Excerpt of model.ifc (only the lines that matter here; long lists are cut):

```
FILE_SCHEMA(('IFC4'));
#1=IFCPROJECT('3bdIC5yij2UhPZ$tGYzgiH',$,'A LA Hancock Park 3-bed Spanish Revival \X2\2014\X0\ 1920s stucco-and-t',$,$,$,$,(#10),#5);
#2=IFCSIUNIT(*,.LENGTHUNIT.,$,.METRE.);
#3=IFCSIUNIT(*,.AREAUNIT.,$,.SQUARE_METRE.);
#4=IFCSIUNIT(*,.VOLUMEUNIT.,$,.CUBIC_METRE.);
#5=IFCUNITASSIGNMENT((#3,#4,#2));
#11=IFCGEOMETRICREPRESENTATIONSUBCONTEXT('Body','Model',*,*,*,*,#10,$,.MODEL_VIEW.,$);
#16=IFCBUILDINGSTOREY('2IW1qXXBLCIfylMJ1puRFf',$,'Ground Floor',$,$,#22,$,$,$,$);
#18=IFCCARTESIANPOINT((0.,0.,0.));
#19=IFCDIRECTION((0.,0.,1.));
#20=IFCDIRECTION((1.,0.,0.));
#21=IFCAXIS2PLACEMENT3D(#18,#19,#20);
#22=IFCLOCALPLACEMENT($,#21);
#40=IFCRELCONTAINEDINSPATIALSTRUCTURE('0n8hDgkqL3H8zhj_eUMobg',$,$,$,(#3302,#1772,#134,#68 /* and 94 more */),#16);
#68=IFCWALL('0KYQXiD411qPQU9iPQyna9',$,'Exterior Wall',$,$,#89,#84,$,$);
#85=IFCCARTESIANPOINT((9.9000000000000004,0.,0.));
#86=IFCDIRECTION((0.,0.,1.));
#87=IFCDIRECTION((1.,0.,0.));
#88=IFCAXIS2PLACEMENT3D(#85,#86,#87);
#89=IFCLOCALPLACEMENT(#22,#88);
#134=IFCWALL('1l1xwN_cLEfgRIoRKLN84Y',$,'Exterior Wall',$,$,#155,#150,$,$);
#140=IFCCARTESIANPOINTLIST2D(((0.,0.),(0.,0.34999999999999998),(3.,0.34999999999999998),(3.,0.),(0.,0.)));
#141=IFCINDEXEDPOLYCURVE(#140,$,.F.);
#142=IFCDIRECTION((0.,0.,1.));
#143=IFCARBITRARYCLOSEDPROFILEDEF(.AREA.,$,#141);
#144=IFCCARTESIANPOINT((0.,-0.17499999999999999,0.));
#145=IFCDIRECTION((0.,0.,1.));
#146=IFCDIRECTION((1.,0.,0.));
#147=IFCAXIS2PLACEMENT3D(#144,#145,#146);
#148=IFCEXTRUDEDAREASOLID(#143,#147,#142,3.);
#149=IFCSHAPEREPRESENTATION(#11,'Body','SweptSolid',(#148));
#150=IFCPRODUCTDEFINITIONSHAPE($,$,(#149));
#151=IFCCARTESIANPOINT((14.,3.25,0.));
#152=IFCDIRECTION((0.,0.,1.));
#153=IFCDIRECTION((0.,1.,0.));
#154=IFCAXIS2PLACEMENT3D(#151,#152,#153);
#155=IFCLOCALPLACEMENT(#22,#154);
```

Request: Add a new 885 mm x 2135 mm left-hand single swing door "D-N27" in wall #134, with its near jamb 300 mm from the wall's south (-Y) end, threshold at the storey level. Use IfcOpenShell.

```python
import numpy as np
import ifcopenshell
import ifcopenshell.api.feature
import ifcopenshell.api.geometry
import ifcopenshell.api.root
import ifcopenshell.api.spatial
import ifcopenshell.geom
import ifcopenshell.util.element
import ifcopenshell.util.placement
import ifcopenshell.util.representation
import ifcopenshell.util.shape
import ifcopenshell.util.unit

model = ifcopenshell.open("model.ifc")
unit_scale = ifcopenshell.util.unit.calculate_unit_scale(model)
settings = ifcopenshell.geom.settings()


def volume(element):
    """Net volume in cubic metres, openings subtracted."""
    shape = ifcopenshell.geom.create_shape(settings, element)
    return ifcopenshell.util.shape.get_volume(shape.geometry)


wall = model.by_guid("1l1xwN_cLEfgRIoRKLN84Y")
storey = ifcopenshell.util.element.get_container(wall, ifc_class="IfcBuildingStorey")
context = ifcopenshell.util.representation.get_context(model, "Model", "Body", "MODEL_VIEW")
before = volume(wall)

width, height, from_end, sill = 0.885, 2.135, 0.3, 0.0  # metres

# The wall runs along its own X axis, and the end named is its -X end.
wall_shape = ifcopenshell.geom.create_shape(settings, wall)
x, y, z = ifcopenshell.util.shape.get_vertices(wall_shape.geometry).T
start = x.min() + from_end
face, thickness = float(y.min()), float(y.max() - y.min())
wall_matrix = ifcopenshell.util.placement.get_local_placement(wall.ObjectPlacement)
level = ifcopenshell.util.placement.get_local_placement(storey.ObjectPlacement)[2, 3]


def in_wall(x, y):
    """Placement at x, y metres in the wall's axes, at sill height."""
    matrix = wall_matrix.copy()
    matrix[:, 3] = wall_matrix @ np.array([x / unit_scale, y / unit_scale, 0.0, 1.0])
    matrix[2, 3] = level + sill / unit_scale
    return matrix


# Opening: a box that overshoots both wall faces by 50 mm.
opening = ifcopenshell.api.root.create_entity(model, ifc_class="IfcOpeningElement", predefined_type="OPENING")
box = ifcopenshell.api.geometry.add_wall_representation(
    model, context=context, length=width, height=height, thickness=thickness + 0.1
)
ifcopenshell.api.geometry.assign_representation(model, product=opening, representation=box)
ifcopenshell.api.geometry.edit_object_placement(model, product=opening, matrix=in_wall(start, face - 0.05), is_si=False)
ifcopenshell.api.feature.add_feature(model, feature=opening, element=wall)

door = ifcopenshell.api.root.create_entity(model, ifc_class="IfcDoor", name="D-N27", predefined_type="DOOR")
door.OverallWidth, door.OverallHeight = width / unit_scale, height / unit_scale
door.OperationType = "SINGLE_SWING_LEFT"
body = ifcopenshell.api.geometry.add_door_representation(
    model,
    context=context,
    overall_width=door.OverallWidth,
    overall_height=door.OverallHeight,
    operation_type="SINGLE_SWING_LEFT",
    lining_properties={"LiningDepth": thickness / unit_scale, "ThresholdDepth": thickness / unit_scale},
)
ifcopenshell.api.geometry.assign_representation(model, product=door, representation=body)
ifcopenshell.api.spatial.assign_container(model, products=[door], relating_structure=storey)
ifcopenshell.api.feature.add_filling(model, opening=opening, element=door)

# The lining spans the wall, so the door starts at the wall face.
ifcopenshell.api.geometry.edit_object_placement(model, product=door, matrix=in_wall(start, face), is_si=False)

after = volume(wall)

print(f"wall volume {before:.3f} -> {after:.3f} m3")

model.write("model-out.ifc")
```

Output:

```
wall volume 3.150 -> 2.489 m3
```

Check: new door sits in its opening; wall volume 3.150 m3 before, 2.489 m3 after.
